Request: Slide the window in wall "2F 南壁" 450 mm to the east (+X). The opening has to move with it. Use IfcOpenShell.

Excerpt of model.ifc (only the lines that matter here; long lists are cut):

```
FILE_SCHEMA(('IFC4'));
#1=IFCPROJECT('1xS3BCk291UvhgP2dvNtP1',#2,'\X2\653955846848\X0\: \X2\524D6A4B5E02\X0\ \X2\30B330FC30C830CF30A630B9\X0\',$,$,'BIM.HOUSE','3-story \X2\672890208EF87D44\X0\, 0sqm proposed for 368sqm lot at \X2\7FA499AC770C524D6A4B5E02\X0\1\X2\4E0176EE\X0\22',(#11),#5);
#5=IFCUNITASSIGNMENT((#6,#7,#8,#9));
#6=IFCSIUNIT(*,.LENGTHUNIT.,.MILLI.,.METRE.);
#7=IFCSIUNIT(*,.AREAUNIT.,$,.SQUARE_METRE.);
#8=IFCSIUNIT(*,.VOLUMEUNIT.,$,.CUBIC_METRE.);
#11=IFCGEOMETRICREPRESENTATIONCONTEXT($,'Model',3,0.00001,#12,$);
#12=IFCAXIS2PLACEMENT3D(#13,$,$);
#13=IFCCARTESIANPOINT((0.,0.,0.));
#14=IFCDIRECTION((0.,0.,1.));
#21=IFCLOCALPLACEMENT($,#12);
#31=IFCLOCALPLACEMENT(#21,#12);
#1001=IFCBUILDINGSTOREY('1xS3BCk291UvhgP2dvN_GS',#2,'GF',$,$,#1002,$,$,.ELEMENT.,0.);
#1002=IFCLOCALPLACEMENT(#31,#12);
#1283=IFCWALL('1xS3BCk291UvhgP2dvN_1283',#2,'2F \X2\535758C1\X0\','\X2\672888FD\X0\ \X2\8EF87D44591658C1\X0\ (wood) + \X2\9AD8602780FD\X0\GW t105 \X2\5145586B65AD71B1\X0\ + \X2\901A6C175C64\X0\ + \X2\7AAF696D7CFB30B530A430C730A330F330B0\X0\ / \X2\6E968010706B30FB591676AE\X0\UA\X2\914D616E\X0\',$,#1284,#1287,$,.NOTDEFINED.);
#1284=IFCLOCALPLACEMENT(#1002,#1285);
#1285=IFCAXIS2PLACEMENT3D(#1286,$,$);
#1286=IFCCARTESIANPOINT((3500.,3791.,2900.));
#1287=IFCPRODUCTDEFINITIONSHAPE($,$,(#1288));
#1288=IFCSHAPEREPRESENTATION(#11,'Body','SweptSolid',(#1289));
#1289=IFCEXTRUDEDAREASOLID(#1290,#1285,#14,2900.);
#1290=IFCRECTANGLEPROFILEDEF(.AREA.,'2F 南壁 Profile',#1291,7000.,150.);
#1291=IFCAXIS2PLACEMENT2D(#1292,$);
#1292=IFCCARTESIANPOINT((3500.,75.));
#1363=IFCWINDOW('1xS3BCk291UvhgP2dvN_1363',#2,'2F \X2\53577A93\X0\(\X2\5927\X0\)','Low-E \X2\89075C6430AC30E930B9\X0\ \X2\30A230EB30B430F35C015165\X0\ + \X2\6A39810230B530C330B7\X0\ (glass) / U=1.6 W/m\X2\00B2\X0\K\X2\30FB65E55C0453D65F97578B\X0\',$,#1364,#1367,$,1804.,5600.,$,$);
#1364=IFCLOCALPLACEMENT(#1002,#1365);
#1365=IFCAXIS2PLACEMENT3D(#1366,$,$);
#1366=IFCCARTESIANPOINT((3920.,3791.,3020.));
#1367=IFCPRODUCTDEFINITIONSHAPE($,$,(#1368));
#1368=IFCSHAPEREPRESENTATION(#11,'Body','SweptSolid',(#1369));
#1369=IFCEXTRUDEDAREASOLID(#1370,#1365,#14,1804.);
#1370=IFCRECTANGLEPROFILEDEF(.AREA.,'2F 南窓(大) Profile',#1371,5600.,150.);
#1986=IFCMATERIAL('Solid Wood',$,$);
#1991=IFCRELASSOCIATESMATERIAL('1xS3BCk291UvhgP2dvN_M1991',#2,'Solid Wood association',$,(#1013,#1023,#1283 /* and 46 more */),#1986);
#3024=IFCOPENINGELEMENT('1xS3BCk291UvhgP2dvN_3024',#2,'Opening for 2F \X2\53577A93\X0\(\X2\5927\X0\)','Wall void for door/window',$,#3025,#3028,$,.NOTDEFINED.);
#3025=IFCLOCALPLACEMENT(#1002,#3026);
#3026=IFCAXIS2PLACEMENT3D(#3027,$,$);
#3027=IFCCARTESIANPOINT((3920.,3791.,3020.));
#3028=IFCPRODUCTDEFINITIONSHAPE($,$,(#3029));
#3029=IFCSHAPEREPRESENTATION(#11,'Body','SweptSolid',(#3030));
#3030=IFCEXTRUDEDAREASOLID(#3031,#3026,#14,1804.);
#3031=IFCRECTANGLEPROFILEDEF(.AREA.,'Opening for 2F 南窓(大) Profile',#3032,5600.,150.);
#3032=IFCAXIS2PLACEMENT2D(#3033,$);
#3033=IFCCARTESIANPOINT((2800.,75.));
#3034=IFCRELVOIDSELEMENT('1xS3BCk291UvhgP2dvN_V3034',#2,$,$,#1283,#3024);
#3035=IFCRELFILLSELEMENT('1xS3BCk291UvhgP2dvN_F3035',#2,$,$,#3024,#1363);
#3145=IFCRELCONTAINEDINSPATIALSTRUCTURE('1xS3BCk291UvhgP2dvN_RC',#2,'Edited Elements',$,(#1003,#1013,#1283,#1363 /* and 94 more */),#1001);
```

```python
import ifcopenshell
import ifcopenshell.api.geometry
import ifcopenshell.util.placement
import ifcopenshell.util.unit

model = ifcopenshell.open("model.ifc")
unit_scale = ifcopenshell.util.unit.calculate_unit_scale(model)

window = model.by_guid("1xS3BCk291UvhgP2dvN_1363")
opening = window.FillsVoids[0].RelatingOpeningElement
wall = opening.VoidsElements[0].RelatingBuildingElement

wall_matrix = ifcopenshell.util.placement.get_local_placement(wall.ObjectPlacement)
shift = wall_matrix[:3, 0] * 0.45 / unit_scale
before = ifcopenshell.util.placement.get_local_placement(window.ObjectPlacement)[:3, 3].copy()

# The window is not placed relative to its opening, so move both.
for product in (opening, window):
    matrix = ifcopenshell.util.placement.get_local_placement(product.ObjectPlacement)
    matrix[:3, 3] += shift
    ifcopenshell.api.geometry.edit_object_placement(model, product=product, matrix=matrix, is_si=False)

after = ifcopenshell.util.placement.get_local_placement(window.ObjectPlacement)[:3, 3]
print("window moved by", (after - before).round(3) + 0.0)

model.write("model_edited.ifc")
```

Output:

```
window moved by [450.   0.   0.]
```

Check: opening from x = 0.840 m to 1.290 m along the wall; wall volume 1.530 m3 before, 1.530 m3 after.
